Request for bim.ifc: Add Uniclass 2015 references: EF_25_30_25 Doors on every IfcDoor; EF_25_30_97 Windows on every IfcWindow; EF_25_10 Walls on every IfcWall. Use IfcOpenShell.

First a look at what the model holds.

```python
import ifcopenshell

model = ifcopenshell.open("bim.ifc")
print(model.schema)
print("classifications:", [c.Name for c in model.by_type("IfcClassification")])
for ifc_class in ("IfcDoor", "IfcRoof", "IfcStair", "IfcWall", "IfcWindow"):
    print(ifc_class, len(model.by_type(ifc_class)))
```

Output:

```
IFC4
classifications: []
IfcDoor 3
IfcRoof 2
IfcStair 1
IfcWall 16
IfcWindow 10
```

```python
import ifcopenshell
import ifcopenshell.api.classification

model = ifcopenshell.open("bim.ifc")

system = ifcopenshell.api.classification.add_classification(model, classification="Uniclass 2015")

codes = {
    "IfcDoor": ("EF_25_30_25", "Doors"),
    "IfcWindow": ("EF_25_30_97", "Windows"),
    "IfcWall": ("EF_25_10", "Walls"),
}
for ifc_class, (code, name) in codes.items():
    products = model.by_type(ifc_class)
    ifcopenshell.api.classification.add_reference(
        model, products=products, classification=system, identification=code, name=name
    )
    print(code, len(products))

model.write("bim_v2.ifc")
```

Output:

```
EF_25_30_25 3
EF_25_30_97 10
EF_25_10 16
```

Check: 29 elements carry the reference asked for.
